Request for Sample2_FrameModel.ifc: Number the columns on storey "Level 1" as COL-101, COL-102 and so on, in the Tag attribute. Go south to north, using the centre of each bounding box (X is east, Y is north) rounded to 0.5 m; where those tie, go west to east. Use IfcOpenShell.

First a look at what the model holds.

```python
import ifcopenshell
import ifcopenshell.util.element
import ifcopenshell.util.placement

model = ifcopenshell.open("Sample2_FrameModel.ifc")
print(model.schema)
storey = next(s for s in model.by_type("IfcBuildingStorey") if s.Name == "Level 1")
columns = [e for e in ifcopenshell.util.element.get_decomposition(storey) if e.is_a("IfcColumn")]
for e in sorted(columns, key=lambda e: e.id()):
    origin = ifcopenshell.util.placement.get_local_placement(e.ObjectPlacement)[:3, 3]
    print(e.id(), e.Tag, e.Name, origin.round(2) + 0.0, sep=" | ")
```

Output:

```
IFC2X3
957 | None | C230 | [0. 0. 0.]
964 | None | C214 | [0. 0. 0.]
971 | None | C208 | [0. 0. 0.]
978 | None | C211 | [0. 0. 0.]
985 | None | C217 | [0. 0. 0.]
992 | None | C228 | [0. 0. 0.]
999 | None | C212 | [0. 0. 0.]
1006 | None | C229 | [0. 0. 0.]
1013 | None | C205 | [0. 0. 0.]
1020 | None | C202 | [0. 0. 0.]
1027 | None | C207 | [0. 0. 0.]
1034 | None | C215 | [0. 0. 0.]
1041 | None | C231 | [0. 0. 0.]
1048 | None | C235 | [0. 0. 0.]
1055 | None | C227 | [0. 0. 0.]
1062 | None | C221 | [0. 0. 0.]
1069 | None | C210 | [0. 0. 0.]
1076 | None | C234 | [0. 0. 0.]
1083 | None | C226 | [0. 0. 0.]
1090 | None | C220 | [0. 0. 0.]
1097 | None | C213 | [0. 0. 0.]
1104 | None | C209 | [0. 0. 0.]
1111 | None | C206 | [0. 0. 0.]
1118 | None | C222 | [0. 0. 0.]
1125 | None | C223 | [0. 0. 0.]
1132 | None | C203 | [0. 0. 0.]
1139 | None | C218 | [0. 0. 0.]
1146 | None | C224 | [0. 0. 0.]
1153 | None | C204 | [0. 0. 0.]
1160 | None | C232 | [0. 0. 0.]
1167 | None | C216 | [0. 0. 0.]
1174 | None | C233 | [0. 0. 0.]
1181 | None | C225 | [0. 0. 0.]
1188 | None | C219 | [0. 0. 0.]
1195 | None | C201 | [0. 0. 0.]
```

```python
import ifcopenshell
import ifcopenshell.geom
import ifcopenshell.util.element
import ifcopenshell.util.shape

model = ifcopenshell.open("Sample2_FrameModel.ifc")
settings = ifcopenshell.geom.settings()
settings.set("use-world-coords", True)


def centre(element):
    shape = ifcopenshell.geom.create_shape(settings, element)
    return ifcopenshell.util.shape.get_bbox_centroid(shape.geometry)


storey = next(s for s in model.by_type("IfcBuildingStorey") if s.Name == "Level 1")
columns = [e for e in ifcopenshell.util.element.get_decomposition(storey) if e.is_a("IfcColumn")]

# Insertion points can sit at a corner or the storey origin, so sort by the geometry (in metres).
centres = {e: centre(e) for e in columns}
columns.sort(key=lambda e: (round(centres[e][1] / 0.5), centres[e][0]))

for i, e in enumerate(columns, start=1):
    number = f"COL-1{i:02d}"
    e.Tag = number
    print(e.id(), number)

model.write("Sample2_FrameModel_v2.ifc")
```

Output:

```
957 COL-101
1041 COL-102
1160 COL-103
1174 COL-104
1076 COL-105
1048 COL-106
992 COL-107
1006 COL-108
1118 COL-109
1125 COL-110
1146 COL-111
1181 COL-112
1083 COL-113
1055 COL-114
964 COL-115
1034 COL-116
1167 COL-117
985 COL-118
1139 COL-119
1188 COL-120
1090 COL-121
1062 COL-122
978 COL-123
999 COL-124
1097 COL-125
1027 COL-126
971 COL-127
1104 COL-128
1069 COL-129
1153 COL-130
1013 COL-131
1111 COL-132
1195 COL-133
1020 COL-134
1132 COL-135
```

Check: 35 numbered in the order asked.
